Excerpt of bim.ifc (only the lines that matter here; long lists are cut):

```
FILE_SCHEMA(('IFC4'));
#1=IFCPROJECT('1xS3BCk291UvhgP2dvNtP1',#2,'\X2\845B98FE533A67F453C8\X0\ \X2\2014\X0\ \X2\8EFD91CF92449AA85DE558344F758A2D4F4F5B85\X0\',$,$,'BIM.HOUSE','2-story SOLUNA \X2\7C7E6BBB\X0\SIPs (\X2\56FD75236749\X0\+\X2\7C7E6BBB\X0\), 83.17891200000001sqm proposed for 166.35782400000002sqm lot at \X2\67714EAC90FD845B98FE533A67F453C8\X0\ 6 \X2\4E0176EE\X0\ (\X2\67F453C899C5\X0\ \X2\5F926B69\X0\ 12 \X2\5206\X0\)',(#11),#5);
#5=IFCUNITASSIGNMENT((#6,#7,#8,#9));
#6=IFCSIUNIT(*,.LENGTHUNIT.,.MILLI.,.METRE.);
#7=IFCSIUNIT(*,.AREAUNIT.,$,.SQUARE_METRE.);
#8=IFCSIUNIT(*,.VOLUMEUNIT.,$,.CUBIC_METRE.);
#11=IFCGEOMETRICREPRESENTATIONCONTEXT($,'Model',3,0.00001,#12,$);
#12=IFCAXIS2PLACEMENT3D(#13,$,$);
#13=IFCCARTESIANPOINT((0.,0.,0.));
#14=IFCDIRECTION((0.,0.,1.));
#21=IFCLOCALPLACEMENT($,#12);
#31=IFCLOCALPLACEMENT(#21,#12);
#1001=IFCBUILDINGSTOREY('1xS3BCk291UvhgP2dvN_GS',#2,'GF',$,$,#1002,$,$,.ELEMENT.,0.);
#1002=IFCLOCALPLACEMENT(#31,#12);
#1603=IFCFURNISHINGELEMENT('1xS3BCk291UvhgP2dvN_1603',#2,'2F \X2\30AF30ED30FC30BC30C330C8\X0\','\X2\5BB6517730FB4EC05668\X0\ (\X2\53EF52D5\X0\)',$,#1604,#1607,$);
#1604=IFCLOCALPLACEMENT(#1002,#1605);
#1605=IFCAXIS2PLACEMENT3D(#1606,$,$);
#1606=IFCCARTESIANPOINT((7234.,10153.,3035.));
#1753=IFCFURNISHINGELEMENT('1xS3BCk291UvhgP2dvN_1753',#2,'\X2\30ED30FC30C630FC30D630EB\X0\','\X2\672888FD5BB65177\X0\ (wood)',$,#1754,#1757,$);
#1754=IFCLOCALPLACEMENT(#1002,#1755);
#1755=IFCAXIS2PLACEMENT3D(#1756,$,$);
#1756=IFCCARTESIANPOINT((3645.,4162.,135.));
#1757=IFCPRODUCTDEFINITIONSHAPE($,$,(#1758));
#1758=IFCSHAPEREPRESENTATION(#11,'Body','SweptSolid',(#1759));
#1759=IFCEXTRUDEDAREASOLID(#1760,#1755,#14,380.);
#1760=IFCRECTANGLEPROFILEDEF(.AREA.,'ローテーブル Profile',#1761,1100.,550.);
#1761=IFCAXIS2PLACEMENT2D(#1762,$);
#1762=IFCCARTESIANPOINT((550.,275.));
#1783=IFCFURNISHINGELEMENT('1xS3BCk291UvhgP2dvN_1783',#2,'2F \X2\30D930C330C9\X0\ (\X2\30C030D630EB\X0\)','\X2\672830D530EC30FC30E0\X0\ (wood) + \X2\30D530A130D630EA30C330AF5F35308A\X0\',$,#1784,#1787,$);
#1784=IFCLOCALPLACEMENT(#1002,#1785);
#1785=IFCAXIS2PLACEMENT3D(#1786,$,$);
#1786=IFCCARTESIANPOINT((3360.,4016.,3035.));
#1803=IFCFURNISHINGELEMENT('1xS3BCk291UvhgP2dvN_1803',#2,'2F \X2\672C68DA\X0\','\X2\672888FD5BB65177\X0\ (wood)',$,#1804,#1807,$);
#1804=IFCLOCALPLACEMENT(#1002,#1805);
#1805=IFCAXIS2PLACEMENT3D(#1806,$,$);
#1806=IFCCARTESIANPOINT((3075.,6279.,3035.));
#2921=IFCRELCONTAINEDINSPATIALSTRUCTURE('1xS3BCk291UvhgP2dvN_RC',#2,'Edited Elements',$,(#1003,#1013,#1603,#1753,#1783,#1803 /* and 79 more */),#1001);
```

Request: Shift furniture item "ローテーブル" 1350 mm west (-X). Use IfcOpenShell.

```python
import ifcopenshell
import ifcopenshell.api.geometry
import ifcopenshell.util.placement
import ifcopenshell.util.unit

model = ifcopenshell.open("bim.ifc")
unit_scale = ifcopenshell.util.unit.calculate_unit_scale(model)

item = model.by_guid("1xS3BCk291UvhgP2dvN_1753")
matrix = ifcopenshell.util.placement.get_local_placement(item.ObjectPlacement)
matrix[0, 3] -= 1.35 / unit_scale
ifcopenshell.api.geometry.edit_object_placement(model, product=item, matrix=matrix, is_si=False)

print(ifcopenshell.util.placement.get_local_placement(item.ObjectPlacement).round(3) + 0.0)

model.write("bim_rev.ifc")
```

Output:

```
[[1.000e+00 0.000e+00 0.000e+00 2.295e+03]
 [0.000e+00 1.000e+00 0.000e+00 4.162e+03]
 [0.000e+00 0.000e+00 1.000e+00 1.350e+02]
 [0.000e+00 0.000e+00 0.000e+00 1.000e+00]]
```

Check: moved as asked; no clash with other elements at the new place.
